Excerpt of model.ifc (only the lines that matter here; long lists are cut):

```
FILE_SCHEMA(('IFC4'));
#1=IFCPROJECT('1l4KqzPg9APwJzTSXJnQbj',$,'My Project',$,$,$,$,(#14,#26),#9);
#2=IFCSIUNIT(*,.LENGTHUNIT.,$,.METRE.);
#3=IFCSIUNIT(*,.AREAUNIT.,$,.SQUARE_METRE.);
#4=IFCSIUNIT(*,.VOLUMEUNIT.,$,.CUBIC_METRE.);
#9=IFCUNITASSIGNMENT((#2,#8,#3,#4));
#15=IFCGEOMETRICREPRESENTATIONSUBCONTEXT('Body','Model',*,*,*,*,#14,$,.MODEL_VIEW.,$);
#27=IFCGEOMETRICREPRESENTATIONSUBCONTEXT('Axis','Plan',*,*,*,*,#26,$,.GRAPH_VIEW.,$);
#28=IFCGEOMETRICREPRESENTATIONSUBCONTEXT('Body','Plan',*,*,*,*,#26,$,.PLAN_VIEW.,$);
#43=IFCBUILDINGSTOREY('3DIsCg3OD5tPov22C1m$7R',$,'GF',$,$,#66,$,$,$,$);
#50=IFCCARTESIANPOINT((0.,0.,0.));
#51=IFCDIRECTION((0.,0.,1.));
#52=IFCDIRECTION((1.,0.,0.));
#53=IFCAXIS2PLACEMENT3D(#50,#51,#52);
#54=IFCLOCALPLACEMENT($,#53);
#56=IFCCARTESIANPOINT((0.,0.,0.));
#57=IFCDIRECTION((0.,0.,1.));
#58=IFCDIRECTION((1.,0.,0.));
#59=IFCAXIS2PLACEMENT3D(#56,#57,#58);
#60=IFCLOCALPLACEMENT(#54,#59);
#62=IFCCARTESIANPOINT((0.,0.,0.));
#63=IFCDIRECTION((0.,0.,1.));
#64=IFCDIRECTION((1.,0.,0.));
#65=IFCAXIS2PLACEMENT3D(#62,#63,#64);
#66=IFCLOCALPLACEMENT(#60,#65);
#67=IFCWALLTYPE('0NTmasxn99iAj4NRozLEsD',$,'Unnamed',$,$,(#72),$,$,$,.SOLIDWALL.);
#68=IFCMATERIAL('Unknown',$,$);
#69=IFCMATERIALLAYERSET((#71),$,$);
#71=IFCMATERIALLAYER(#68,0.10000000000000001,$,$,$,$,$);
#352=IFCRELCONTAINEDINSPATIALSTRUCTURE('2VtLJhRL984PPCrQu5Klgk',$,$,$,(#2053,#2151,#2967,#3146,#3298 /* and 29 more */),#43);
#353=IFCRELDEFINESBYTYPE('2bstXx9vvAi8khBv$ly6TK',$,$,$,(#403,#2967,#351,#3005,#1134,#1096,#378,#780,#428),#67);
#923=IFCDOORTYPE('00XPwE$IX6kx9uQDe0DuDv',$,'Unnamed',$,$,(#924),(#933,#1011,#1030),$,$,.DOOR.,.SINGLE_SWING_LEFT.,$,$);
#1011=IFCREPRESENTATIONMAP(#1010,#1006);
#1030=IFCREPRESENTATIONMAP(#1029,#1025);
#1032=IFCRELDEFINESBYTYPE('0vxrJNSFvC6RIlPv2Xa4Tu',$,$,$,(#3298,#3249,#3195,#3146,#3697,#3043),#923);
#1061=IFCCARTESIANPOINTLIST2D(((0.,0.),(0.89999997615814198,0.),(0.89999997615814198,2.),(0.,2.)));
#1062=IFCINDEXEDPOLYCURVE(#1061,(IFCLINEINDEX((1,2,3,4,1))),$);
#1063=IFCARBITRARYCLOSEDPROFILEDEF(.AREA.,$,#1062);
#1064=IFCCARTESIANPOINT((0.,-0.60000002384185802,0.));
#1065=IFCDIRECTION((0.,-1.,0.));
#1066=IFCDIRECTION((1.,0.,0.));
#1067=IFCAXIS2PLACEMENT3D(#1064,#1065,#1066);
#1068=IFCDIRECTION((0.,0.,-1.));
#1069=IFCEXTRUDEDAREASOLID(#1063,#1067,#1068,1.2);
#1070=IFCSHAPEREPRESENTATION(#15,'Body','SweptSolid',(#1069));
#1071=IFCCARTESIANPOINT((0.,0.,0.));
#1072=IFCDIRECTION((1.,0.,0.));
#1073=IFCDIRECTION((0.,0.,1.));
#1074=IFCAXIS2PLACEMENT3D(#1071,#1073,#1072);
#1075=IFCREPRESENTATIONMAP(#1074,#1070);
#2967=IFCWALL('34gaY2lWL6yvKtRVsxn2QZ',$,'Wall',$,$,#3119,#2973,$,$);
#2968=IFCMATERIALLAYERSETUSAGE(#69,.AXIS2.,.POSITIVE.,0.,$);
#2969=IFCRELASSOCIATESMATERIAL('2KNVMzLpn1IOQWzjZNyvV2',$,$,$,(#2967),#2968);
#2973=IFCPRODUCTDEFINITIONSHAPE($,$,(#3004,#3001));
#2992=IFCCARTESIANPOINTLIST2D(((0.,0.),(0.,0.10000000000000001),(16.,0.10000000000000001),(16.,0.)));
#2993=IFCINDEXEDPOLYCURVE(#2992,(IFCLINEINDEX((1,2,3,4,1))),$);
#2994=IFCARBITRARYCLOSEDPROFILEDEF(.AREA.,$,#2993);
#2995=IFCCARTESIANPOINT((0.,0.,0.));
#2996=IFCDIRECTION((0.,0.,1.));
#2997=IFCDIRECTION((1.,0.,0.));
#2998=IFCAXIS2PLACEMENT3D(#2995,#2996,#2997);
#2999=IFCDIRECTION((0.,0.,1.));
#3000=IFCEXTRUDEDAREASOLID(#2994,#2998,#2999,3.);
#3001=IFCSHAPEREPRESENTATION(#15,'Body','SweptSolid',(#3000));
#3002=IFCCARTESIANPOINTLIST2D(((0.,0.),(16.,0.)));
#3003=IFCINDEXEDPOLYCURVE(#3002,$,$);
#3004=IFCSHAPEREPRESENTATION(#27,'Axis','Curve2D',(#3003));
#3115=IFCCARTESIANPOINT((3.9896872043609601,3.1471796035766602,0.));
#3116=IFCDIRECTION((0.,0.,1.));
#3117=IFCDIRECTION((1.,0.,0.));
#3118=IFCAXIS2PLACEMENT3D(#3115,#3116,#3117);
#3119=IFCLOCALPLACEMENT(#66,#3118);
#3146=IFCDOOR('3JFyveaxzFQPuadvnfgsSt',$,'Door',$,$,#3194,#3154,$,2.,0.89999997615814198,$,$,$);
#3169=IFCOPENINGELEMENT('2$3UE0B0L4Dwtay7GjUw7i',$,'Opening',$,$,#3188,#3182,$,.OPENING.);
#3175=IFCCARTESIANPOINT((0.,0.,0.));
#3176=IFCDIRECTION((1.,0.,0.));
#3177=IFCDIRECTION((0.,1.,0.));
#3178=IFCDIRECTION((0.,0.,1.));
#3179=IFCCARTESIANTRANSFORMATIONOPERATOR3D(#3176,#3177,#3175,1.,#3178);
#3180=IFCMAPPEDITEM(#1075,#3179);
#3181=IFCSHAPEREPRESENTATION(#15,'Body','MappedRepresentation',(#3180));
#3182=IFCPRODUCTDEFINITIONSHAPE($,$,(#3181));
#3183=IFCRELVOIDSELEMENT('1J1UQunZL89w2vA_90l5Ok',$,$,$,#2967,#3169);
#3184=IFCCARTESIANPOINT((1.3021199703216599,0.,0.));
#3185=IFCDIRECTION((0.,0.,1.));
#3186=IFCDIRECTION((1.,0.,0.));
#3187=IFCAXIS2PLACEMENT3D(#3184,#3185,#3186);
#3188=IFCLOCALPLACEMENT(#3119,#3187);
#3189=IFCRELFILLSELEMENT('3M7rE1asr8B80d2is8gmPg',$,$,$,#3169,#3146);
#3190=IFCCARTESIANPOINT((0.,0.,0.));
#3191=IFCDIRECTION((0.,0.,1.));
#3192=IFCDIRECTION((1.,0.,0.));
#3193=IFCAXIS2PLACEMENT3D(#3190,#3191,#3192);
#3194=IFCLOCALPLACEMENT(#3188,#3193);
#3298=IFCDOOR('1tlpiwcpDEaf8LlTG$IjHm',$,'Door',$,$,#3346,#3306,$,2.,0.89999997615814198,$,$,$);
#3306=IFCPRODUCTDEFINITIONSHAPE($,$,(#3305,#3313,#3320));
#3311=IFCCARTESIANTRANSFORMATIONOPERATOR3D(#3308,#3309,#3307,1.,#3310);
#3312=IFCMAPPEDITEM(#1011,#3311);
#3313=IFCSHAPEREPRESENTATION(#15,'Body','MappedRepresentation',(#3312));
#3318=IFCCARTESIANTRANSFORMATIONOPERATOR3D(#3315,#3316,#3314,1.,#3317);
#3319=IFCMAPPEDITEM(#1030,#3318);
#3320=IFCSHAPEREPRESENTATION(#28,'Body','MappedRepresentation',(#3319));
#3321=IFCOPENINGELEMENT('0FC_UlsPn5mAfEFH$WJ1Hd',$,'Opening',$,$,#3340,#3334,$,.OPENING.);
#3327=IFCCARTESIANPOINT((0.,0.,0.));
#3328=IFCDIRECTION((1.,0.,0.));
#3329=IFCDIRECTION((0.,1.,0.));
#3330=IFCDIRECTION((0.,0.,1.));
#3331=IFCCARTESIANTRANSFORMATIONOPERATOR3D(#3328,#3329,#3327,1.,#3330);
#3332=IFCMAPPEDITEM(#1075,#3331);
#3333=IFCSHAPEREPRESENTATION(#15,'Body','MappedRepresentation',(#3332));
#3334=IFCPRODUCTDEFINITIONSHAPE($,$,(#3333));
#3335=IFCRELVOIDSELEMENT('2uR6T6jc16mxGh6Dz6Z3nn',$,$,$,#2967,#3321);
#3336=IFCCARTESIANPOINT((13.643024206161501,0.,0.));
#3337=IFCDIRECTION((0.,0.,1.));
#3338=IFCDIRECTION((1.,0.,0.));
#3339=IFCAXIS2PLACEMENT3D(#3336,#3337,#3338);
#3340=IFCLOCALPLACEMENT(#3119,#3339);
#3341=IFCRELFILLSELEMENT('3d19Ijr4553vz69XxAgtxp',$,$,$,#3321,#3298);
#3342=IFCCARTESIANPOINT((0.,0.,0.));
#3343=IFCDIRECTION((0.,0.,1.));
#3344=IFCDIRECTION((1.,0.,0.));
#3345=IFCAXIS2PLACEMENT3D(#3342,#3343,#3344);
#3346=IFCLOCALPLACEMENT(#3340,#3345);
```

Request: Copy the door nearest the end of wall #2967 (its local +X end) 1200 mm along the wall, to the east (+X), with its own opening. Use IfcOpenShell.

```python
import ifcopenshell
import ifcopenshell.api.feature
import ifcopenshell.api.geometry
import ifcopenshell.api.root
import ifcopenshell.geom
import ifcopenshell.util.element
import ifcopenshell.util.placement
import ifcopenshell.util.shape

model = ifcopenshell.open("model.ifc")
settings = ifcopenshell.geom.settings()


def volume(element):
    """Net volume in cubic metres, openings subtracted."""
    shape = ifcopenshell.geom.create_shape(settings, element)
    return ifcopenshell.util.shape.get_volume(shape.geometry)


door = model.by_id(3298)
opening = door.FillsVoids[0].RelatingOpeningElement
wall = opening.VoidsElements[0].RelatingBuildingElement
before = volume(wall)
shift = ifcopenshell.util.placement.get_local_placement(wall.ObjectPlacement)[:3, 0] * 1.2

# copy_class copies the void relationship, type, container and properties, but no geometry.
new_opening = ifcopenshell.api.root.copy_class(model, product=opening)
new_opening.Representation = ifcopenshell.util.element.copy_deep(
    model, opening.Representation, exclude=["IfcGeometricRepresentationContext", "IfcRepresentationMap"]
)
new_door = ifcopenshell.api.root.copy_class(model, product=door)
new_door.Representation = ifcopenshell.util.element.copy_deep(
    model, door.Representation, exclude=["IfcGeometricRepresentationContext", "IfcRepresentationMap"]
)
ifcopenshell.api.feature.add_filling(model, opening=new_opening, element=new_door)

for old, new in ((opening, new_opening), (door, new_door)):
    matrix = ifcopenshell.util.placement.get_local_placement(old.ObjectPlacement)
    matrix[:3, 3] += shift
    ifcopenshell.api.geometry.edit_object_placement(model, product=new, matrix=matrix, is_si=False)

after = volume(wall)

print(f"wall volume {before:.3f} -> {after:.3f} m3")

model.write("model_updated.ifc")
```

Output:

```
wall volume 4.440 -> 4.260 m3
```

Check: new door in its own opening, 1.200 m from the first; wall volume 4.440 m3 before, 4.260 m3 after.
